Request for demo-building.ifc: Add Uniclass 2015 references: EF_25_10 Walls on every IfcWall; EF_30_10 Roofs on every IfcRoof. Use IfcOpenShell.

First a look at what the model holds.

```python
import ifcopenshell

model = ifcopenshell.open("demo-building.ifc")
print(model.schema)
print("classifications:", [c.Name for c in model.by_type("IfcClassification")])
for ifc_class in ("IfcDoor", "IfcRoof", "IfcStair", "IfcWall", "IfcWindow"):
    print(ifc_class, len(model.by_type(ifc_class)))
```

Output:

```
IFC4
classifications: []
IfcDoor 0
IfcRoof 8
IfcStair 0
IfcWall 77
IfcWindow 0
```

```python
import ifcopenshell
import ifcopenshell.api.classification

model = ifcopenshell.open("demo-building.ifc")

system = ifcopenshell.api.classification.add_classification(model, classification="Uniclass 2015")

codes = {
    "IfcWall": ("EF_25_10", "Walls"),
    "IfcRoof": ("EF_30_10", "Roofs"),
}
for ifc_class, (code, name) in codes.items():
    products = model.by_type(ifc_class)
    ifcopenshell.api.classification.add_reference(
        model, products=products, classification=system, identification=code, name=name
    )
    print(code, len(products))

model.write("demo-building_edited.ifc")
```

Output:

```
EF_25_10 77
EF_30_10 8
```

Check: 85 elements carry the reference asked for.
